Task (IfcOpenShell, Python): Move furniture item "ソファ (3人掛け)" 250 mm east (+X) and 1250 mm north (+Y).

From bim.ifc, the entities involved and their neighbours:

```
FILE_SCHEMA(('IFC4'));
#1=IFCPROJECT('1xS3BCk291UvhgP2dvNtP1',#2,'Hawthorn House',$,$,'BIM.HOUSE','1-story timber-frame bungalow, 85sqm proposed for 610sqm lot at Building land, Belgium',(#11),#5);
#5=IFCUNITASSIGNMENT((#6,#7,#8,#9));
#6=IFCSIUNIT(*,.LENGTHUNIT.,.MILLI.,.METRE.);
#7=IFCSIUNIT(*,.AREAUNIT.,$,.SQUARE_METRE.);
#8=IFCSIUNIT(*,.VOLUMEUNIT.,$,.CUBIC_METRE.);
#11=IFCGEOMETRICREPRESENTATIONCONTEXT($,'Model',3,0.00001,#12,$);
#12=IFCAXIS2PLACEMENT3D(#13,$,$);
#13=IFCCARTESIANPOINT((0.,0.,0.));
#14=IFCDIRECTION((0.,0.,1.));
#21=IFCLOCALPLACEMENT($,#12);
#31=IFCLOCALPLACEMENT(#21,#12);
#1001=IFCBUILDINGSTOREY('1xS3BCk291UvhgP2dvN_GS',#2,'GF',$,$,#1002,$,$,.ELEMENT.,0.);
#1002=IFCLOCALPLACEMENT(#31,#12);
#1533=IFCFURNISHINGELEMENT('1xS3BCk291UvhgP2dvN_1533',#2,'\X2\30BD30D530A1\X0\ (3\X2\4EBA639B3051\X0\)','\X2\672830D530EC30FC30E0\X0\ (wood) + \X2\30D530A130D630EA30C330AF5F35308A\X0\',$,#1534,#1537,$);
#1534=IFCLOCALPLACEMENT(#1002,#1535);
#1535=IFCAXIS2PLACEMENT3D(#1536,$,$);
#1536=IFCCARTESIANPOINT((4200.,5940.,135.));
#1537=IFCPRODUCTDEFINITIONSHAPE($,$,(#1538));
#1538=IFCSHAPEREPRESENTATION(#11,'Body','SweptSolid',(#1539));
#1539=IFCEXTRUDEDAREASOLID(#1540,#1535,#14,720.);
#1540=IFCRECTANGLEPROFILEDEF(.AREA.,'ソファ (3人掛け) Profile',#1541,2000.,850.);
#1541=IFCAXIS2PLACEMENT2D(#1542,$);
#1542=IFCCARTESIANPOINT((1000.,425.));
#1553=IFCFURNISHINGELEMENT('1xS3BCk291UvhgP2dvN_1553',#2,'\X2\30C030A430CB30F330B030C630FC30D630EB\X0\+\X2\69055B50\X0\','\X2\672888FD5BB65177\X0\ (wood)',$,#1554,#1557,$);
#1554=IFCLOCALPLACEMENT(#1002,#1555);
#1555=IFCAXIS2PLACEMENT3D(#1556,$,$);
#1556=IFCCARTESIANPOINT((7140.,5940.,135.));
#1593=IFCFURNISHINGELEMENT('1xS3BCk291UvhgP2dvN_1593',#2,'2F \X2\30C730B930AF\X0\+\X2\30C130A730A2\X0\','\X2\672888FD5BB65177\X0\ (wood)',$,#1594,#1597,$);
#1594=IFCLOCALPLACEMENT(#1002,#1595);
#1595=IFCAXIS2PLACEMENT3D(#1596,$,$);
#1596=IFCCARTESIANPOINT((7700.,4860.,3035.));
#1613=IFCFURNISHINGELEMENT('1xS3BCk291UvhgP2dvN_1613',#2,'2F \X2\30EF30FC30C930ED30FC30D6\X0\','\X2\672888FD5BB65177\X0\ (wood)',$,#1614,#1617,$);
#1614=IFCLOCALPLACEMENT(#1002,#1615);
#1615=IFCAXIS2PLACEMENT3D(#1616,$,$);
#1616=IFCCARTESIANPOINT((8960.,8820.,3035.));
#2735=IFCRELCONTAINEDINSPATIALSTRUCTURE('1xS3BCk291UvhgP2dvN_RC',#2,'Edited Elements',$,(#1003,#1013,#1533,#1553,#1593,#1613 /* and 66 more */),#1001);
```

```python
import ifcopenshell
import ifcopenshell.api.geometry
import ifcopenshell.util.placement
import ifcopenshell.util.unit

model = ifcopenshell.open("bim.ifc")
unit_scale = ifcopenshell.util.unit.calculate_unit_scale(model)

item = model.by_guid("1xS3BCk291UvhgP2dvN_1533")
matrix = ifcopenshell.util.placement.get_local_placement(item.ObjectPlacement)
matrix[0, 3] += 0.25 / unit_scale
matrix[1, 3] += 1.25 / unit_scale
ifcopenshell.api.geometry.edit_object_placement(model, product=item, matrix=matrix, is_si=False)

print(ifcopenshell.util.placement.get_local_placement(item.ObjectPlacement).round(3) + 0.0)

model.write("bim_updated.ifc")
```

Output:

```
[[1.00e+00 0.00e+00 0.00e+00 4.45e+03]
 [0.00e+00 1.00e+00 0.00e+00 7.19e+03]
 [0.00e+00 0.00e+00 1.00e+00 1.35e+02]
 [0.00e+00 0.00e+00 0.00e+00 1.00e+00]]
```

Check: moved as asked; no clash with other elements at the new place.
